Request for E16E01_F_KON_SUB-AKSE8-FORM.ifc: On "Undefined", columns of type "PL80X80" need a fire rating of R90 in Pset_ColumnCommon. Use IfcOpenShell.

First a look at what the model holds.

```python
import ifcopenshell
import ifcopenshell.util.element

model = ifcopenshell.open("E16E01_F_KON_SUB-AKSE8-FORM.ifc")
print(model.schema)
storey = next(s for s in model.by_type("IfcBuildingStorey") if s.Name == "Undefined")
columns = [e for e in ifcopenshell.util.element.get_decomposition(storey) if e.is_a("IfcColumn")]
seen = {}
for e in columns:
    element_type = ifcopenshell.util.element.get_type(e)
    key = (element_type.Name if element_type != e and element_type else None, ifcopenshell.util.element.get_pset(e, "Pset_ColumnCommon", "FireRating"))
    seen[key] = seen.get(key, 0) + 1
for (name, value), count in sorted(seen.items(), key=str):
    print(count, "x", name, "|", value)
```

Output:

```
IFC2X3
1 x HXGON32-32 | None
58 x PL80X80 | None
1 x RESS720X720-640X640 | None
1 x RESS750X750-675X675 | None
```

```python
import ifcopenshell
import ifcopenshell.api.pset
import ifcopenshell.util.element

model = ifcopenshell.open("E16E01_F_KON_SUB-AKSE8-FORM.ifc")

storey = next(s for s in model.by_type("IfcBuildingStorey") if s.Name == "Undefined")
columns = [e for e in ifcopenshell.util.element.get_decomposition(storey) if e.is_a("IfcColumn")]

count = 0
for e in columns:
    element_type = ifcopenshell.util.element.get_type(e)
    if element_type in (None, e) or element_type.Name != "PL80X80":
        continue
    found = ifcopenshell.util.element.get_pset(e, "Pset_ColumnCommon", should_inherit=False)
    if found:
        pset = model.by_id(found["id"])
        if len(ifcopenshell.util.element.get_elements_by_pset(pset)) > 1:
            pset = ifcopenshell.api.pset.unshare_pset(model, products=[e], pset=pset)[0]
    else:
        pset = ifcopenshell.api.pset.add_pset(model, product=e, name="Pset_ColumnCommon")
    ifcopenshell.api.pset.edit_pset(model, pset=pset, properties={"FireRating": "R90"})
    count += 1

print(count, "columns updated")

model.write("E16E01_F_KON_SUB-AKSE8-FORM_rev.ifc")
```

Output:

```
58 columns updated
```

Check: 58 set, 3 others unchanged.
